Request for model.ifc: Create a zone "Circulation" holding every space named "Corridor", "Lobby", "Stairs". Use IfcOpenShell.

First a look at what the model holds.

```python
import ifcopenshell

model = ifcopenshell.open("model.ifc")
print(model.schema)
seen = {}
for space in model.by_type("IfcSpace"):
    seen[space.LongName] = seen.get(space.LongName, 0) + 1
for name, count in sorted(seen.items(), key=str):
    print(count, "x", name)
print("zones:", [z.Name for z in model.by_type("IfcZone")][:20])
```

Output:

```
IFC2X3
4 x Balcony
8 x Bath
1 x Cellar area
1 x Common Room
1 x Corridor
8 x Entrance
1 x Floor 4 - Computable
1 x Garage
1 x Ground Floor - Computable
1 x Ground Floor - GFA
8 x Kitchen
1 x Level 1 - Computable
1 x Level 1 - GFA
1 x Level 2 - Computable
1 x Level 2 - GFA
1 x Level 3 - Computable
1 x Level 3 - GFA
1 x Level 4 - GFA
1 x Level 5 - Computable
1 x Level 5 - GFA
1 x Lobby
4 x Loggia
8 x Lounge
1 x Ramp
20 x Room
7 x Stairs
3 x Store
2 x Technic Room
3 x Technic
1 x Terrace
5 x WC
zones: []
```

```python
import ifcopenshell
import ifcopenshell.api.group
import ifcopenshell.api.root

model = ifcopenshell.open("model.ifc")

names = {"Corridor", "Lobby", "Stairs"}
spaces = [s for s in model.by_type("IfcSpace") if s.LongName in names]

zone = ifcopenshell.api.root.create_entity(model, ifc_class="IfcZone", name="Circulation")
ifcopenshell.api.group.assign_group(model, products=spaces, group=zone)
print(len(spaces), "spaces in", zone.Name)

model.write("model_updated.ifc")
```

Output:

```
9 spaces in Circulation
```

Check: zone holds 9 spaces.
